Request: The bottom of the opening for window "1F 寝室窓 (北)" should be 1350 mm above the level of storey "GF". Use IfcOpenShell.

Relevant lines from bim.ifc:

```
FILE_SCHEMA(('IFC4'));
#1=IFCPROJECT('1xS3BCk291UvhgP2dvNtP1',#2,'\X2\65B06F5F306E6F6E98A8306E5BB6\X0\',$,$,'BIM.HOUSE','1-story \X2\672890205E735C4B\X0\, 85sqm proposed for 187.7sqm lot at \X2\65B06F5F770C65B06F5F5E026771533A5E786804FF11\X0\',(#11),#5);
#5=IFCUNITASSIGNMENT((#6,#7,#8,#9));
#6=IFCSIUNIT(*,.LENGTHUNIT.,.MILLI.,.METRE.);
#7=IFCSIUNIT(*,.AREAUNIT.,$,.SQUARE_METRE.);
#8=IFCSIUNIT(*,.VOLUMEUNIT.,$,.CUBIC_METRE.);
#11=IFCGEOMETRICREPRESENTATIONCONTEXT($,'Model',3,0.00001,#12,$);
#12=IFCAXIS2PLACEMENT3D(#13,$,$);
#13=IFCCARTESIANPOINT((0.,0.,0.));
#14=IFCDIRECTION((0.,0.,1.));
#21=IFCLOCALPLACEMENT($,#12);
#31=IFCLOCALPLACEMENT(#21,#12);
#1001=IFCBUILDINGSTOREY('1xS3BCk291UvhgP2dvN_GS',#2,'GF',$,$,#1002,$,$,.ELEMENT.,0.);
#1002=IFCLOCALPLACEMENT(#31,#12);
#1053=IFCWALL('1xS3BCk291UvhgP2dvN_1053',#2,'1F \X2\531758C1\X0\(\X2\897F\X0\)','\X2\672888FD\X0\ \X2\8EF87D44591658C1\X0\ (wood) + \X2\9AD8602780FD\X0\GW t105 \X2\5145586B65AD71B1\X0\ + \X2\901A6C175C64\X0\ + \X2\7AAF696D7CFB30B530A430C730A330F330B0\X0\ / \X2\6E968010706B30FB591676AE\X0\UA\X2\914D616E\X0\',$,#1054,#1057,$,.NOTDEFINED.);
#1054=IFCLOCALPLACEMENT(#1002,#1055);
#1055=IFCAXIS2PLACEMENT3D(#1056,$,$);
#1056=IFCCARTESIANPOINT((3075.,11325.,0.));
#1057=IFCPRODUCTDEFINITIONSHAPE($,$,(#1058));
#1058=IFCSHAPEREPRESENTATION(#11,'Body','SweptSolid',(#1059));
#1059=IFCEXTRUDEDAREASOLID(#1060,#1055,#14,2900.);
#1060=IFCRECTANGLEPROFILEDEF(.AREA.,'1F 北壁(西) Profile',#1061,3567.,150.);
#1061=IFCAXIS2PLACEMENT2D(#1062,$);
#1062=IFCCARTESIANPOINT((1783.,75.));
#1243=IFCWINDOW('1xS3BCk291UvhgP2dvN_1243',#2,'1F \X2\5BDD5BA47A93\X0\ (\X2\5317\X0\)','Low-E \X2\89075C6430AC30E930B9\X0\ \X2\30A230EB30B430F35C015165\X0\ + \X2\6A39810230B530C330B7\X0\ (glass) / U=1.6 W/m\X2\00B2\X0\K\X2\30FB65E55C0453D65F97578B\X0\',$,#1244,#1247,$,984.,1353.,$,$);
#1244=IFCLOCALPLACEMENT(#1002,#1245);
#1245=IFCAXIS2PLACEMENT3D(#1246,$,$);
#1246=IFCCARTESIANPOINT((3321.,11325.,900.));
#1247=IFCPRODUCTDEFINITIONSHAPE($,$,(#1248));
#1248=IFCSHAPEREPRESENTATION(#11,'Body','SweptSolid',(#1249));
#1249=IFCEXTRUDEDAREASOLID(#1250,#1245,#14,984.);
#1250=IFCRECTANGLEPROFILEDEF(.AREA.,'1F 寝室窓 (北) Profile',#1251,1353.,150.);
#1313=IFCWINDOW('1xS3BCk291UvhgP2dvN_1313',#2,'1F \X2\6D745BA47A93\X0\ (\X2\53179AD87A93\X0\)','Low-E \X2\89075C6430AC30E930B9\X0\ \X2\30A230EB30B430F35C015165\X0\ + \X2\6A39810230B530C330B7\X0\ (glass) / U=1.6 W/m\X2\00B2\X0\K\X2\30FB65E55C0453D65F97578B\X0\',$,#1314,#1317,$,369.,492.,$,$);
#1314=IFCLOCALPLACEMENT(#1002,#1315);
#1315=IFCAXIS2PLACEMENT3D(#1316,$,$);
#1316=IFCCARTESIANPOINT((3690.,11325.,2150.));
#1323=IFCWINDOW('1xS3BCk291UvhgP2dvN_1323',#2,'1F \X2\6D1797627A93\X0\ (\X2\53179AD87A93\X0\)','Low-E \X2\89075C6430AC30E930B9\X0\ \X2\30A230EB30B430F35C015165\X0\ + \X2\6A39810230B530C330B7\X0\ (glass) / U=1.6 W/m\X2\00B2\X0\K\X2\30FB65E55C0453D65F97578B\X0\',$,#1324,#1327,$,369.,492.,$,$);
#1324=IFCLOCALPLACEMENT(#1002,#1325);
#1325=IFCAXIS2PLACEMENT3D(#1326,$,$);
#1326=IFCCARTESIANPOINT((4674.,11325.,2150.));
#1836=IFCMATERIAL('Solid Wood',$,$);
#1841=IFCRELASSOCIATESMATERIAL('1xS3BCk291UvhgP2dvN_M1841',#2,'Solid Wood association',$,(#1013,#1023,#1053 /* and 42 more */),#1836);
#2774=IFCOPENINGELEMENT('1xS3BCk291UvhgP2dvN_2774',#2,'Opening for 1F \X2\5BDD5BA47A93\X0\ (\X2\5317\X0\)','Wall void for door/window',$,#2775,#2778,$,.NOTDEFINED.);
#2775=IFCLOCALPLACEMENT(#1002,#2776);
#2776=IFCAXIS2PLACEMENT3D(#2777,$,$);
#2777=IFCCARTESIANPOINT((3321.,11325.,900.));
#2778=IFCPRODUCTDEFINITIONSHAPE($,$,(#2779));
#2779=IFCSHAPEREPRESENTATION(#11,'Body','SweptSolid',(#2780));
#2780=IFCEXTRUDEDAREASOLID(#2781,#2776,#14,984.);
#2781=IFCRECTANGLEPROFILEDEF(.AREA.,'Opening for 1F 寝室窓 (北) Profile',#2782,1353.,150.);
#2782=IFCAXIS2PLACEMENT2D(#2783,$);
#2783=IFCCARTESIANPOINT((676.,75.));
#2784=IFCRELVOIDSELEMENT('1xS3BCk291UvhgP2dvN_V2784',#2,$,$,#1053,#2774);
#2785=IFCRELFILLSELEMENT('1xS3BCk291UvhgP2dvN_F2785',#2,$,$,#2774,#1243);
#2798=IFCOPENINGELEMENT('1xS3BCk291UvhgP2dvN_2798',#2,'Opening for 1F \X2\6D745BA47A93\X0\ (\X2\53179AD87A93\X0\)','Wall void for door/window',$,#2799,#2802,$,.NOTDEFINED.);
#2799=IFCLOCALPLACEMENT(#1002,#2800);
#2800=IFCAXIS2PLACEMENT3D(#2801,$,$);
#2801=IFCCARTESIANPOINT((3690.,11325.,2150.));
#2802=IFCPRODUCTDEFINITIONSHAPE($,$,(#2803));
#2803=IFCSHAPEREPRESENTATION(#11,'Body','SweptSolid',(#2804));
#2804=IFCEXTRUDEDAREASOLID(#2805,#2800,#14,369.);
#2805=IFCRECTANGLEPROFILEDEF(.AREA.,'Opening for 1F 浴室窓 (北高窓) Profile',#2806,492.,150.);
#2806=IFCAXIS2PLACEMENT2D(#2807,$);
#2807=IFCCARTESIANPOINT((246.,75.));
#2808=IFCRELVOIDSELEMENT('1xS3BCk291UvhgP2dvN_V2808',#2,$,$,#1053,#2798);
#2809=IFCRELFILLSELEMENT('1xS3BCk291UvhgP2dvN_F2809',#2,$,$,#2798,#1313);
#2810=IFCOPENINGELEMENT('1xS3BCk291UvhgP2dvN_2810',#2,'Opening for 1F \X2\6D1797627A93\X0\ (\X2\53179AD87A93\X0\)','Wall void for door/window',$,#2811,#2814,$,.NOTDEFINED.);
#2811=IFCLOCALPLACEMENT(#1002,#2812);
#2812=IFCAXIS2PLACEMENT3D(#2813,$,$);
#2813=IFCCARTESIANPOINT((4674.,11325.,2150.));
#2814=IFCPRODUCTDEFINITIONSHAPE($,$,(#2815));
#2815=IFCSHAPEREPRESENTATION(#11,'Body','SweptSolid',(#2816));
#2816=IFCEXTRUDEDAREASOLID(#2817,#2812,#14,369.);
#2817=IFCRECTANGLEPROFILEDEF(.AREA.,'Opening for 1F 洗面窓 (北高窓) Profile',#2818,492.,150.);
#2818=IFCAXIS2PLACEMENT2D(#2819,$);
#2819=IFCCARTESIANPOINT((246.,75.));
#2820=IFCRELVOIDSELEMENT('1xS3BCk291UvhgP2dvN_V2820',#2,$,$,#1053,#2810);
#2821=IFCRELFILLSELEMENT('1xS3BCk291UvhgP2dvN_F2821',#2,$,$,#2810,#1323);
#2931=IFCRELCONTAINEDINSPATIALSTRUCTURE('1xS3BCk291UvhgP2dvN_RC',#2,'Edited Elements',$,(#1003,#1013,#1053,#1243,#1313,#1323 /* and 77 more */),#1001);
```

```python
import numpy as np
import ifcopenshell
import ifcopenshell.api.geometry
import ifcopenshell.geom
import ifcopenshell.util.element
import ifcopenshell.util.placement
import ifcopenshell.util.shape
import ifcopenshell.util.unit

model = ifcopenshell.open("bim.ifc")
unit_scale = ifcopenshell.util.unit.calculate_unit_scale(model)

window = model.by_guid("1xS3BCk291UvhgP2dvN_1243")
opening = window.FillsVoids[0].RelatingOpeningElement
storey = ifcopenshell.util.element.get_container(window, ifc_class="IfcBuildingStorey")
level = ifcopenshell.util.placement.get_local_placement(storey.ObjectPlacement)[2, 3]

# The opening's origin need not be at the sill, so measure its lowest point.
shape = ifcopenshell.geom.create_shape(ifcopenshell.geom.settings(), opening)
bottom = ifcopenshell.util.shape.get_shape_bottom_elevation(shape, shape.geometry) / unit_scale
dz = level + 1.35 / unit_scale - bottom

shift = np.array([0.0, 0.0, dz])
# The window is not placed relative to its opening, so move both.
for product in (opening, window):
    matrix = ifcopenshell.util.placement.get_local_placement(product.ObjectPlacement)
    matrix[:3, 3] += shift
    ifcopenshell.api.geometry.edit_object_placement(model, product=product, matrix=matrix, is_si=False)

print(f"moved by {dz * unit_scale:+.3f} m")

model.write("bim_edited.ifc")
```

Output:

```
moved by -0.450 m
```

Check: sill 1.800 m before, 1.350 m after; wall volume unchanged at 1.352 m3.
